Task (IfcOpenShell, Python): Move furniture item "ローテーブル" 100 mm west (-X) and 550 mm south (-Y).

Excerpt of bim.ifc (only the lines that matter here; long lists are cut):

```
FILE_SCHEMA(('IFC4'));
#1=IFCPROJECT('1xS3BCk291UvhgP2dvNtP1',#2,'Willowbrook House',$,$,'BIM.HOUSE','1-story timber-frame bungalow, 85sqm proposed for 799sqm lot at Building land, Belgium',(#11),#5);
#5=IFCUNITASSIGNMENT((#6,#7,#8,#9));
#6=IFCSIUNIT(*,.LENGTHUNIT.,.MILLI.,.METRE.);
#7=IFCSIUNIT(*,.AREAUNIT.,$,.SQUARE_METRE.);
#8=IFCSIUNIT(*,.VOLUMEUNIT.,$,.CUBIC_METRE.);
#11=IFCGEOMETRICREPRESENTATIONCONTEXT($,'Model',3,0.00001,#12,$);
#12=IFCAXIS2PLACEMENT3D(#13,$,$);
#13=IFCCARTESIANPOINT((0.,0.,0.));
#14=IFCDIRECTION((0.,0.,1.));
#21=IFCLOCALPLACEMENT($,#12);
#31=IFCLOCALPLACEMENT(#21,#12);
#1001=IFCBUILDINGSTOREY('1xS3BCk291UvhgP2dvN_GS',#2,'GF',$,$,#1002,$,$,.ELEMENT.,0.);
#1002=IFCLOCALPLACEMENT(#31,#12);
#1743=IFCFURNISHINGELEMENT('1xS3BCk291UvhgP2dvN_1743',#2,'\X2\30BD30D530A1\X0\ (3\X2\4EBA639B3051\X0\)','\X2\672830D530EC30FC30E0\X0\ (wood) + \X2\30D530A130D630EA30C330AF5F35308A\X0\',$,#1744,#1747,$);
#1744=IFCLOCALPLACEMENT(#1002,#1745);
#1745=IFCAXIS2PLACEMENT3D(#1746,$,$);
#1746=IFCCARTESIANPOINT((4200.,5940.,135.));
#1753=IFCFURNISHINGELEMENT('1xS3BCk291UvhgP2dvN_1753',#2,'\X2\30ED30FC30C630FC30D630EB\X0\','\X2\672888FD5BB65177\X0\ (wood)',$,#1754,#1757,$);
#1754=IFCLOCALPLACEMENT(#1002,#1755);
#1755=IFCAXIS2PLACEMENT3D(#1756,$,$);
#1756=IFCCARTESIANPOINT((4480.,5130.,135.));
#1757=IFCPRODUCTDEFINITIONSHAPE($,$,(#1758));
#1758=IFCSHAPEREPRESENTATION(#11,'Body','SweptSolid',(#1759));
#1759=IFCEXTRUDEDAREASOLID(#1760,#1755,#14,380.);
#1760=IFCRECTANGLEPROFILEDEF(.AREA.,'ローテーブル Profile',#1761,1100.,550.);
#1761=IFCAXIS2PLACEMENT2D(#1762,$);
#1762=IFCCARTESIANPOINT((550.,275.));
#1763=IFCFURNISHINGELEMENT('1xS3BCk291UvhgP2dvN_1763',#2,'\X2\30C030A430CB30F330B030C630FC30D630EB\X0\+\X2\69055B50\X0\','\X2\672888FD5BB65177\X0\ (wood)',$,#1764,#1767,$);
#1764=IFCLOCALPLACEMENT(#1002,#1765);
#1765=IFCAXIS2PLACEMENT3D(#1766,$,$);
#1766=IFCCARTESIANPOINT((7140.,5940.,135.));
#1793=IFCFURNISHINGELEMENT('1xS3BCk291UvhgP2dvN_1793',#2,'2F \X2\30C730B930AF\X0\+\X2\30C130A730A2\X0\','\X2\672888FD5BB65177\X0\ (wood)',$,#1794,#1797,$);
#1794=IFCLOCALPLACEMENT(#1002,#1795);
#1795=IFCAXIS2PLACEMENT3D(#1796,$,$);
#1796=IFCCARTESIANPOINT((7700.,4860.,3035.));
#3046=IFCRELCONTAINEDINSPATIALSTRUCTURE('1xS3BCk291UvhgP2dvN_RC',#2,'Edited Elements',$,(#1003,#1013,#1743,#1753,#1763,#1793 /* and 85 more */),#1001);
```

```python
import ifcopenshell
import ifcopenshell.api.geometry
import ifcopenshell.util.placement
import ifcopenshell.util.unit

model = ifcopenshell.open("bim.ifc")
unit_scale = ifcopenshell.util.unit.calculate_unit_scale(model)

item = model.by_guid("1xS3BCk291UvhgP2dvN_1753")
matrix = ifcopenshell.util.placement.get_local_placement(item.ObjectPlacement)
matrix[0, 3] -= 0.1 / unit_scale
matrix[1, 3] -= 0.55 / unit_scale
ifcopenshell.api.geometry.edit_object_placement(model, product=item, matrix=matrix, is_si=False)

print(ifcopenshell.util.placement.get_local_placement(item.ObjectPlacement).round(3) + 0.0)

model.write("bim-out.ifc")
```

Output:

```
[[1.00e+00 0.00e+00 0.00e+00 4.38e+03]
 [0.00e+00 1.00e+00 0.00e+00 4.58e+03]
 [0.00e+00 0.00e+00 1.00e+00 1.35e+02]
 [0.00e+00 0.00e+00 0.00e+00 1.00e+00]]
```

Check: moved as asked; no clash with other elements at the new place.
